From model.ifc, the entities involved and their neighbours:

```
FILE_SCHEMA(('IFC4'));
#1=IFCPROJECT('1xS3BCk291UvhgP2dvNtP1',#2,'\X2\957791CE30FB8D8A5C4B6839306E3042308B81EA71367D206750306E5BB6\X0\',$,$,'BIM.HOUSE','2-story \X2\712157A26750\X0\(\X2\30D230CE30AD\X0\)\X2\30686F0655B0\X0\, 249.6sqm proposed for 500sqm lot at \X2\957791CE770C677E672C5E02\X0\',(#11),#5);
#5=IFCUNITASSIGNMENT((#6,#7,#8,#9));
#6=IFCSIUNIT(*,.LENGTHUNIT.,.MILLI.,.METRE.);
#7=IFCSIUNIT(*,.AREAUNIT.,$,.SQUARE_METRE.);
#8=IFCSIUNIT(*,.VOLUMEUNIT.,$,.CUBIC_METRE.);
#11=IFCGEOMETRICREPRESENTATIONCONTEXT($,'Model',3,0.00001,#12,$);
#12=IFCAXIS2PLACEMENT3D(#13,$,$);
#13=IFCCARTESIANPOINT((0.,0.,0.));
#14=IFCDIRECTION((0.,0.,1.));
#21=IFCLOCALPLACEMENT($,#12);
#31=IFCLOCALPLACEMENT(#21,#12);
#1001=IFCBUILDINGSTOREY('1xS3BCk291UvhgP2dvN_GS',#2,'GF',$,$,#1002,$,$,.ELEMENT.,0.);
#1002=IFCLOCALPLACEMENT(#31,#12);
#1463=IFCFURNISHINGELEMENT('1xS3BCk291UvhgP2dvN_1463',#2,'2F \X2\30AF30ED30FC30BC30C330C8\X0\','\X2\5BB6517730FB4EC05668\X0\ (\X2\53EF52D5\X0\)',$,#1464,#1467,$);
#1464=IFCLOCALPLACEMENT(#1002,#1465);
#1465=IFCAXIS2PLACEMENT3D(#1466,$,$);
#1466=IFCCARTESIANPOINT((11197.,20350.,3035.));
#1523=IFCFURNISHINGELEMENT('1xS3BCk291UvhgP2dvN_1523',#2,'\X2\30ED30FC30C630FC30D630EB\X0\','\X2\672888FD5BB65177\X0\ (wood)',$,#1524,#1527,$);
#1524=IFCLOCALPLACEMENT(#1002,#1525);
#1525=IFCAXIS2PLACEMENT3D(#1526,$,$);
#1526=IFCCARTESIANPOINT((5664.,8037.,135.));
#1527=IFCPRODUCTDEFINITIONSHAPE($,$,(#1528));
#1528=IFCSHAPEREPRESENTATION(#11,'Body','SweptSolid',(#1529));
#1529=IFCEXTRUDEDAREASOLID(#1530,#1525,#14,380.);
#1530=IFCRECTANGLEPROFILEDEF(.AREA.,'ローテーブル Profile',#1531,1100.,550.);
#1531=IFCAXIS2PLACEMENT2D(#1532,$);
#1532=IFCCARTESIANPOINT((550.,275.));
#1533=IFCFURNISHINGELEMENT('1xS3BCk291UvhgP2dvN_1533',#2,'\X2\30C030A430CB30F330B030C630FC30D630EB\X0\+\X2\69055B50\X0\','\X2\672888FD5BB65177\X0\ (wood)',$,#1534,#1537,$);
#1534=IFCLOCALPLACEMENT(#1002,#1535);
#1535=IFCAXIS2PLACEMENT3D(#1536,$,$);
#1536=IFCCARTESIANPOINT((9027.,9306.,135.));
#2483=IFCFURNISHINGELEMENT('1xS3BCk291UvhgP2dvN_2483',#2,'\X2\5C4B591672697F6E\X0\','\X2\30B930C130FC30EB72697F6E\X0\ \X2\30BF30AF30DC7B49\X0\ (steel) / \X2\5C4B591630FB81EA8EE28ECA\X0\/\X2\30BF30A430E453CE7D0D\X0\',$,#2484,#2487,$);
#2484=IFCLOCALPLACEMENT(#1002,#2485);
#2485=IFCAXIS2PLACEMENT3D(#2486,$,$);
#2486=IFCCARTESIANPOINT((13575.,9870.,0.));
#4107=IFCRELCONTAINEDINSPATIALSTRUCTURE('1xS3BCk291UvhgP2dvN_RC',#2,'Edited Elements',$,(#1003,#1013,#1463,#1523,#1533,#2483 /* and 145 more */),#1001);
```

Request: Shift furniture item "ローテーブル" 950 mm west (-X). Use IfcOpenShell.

```python
import ifcopenshell
import ifcopenshell.api.geometry
import ifcopenshell.util.placement
import ifcopenshell.util.unit

model = ifcopenshell.open("model.ifc")
unit_scale = ifcopenshell.util.unit.calculate_unit_scale(model)

item = model.by_guid("1xS3BCk291UvhgP2dvN_1523")
matrix = ifcopenshell.util.placement.get_local_placement(item.ObjectPlacement)
matrix[0, 3] -= 0.95 / unit_scale
ifcopenshell.api.geometry.edit_object_placement(model, product=item, matrix=matrix, is_si=False)

print(ifcopenshell.util.placement.get_local_placement(item.ObjectPlacement).round(3) + 0.0)

model.write("model_v2.ifc")
```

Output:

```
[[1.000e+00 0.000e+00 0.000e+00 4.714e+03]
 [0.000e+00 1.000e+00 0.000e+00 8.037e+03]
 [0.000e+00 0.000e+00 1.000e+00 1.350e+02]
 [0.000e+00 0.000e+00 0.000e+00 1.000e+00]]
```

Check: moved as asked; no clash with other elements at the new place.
